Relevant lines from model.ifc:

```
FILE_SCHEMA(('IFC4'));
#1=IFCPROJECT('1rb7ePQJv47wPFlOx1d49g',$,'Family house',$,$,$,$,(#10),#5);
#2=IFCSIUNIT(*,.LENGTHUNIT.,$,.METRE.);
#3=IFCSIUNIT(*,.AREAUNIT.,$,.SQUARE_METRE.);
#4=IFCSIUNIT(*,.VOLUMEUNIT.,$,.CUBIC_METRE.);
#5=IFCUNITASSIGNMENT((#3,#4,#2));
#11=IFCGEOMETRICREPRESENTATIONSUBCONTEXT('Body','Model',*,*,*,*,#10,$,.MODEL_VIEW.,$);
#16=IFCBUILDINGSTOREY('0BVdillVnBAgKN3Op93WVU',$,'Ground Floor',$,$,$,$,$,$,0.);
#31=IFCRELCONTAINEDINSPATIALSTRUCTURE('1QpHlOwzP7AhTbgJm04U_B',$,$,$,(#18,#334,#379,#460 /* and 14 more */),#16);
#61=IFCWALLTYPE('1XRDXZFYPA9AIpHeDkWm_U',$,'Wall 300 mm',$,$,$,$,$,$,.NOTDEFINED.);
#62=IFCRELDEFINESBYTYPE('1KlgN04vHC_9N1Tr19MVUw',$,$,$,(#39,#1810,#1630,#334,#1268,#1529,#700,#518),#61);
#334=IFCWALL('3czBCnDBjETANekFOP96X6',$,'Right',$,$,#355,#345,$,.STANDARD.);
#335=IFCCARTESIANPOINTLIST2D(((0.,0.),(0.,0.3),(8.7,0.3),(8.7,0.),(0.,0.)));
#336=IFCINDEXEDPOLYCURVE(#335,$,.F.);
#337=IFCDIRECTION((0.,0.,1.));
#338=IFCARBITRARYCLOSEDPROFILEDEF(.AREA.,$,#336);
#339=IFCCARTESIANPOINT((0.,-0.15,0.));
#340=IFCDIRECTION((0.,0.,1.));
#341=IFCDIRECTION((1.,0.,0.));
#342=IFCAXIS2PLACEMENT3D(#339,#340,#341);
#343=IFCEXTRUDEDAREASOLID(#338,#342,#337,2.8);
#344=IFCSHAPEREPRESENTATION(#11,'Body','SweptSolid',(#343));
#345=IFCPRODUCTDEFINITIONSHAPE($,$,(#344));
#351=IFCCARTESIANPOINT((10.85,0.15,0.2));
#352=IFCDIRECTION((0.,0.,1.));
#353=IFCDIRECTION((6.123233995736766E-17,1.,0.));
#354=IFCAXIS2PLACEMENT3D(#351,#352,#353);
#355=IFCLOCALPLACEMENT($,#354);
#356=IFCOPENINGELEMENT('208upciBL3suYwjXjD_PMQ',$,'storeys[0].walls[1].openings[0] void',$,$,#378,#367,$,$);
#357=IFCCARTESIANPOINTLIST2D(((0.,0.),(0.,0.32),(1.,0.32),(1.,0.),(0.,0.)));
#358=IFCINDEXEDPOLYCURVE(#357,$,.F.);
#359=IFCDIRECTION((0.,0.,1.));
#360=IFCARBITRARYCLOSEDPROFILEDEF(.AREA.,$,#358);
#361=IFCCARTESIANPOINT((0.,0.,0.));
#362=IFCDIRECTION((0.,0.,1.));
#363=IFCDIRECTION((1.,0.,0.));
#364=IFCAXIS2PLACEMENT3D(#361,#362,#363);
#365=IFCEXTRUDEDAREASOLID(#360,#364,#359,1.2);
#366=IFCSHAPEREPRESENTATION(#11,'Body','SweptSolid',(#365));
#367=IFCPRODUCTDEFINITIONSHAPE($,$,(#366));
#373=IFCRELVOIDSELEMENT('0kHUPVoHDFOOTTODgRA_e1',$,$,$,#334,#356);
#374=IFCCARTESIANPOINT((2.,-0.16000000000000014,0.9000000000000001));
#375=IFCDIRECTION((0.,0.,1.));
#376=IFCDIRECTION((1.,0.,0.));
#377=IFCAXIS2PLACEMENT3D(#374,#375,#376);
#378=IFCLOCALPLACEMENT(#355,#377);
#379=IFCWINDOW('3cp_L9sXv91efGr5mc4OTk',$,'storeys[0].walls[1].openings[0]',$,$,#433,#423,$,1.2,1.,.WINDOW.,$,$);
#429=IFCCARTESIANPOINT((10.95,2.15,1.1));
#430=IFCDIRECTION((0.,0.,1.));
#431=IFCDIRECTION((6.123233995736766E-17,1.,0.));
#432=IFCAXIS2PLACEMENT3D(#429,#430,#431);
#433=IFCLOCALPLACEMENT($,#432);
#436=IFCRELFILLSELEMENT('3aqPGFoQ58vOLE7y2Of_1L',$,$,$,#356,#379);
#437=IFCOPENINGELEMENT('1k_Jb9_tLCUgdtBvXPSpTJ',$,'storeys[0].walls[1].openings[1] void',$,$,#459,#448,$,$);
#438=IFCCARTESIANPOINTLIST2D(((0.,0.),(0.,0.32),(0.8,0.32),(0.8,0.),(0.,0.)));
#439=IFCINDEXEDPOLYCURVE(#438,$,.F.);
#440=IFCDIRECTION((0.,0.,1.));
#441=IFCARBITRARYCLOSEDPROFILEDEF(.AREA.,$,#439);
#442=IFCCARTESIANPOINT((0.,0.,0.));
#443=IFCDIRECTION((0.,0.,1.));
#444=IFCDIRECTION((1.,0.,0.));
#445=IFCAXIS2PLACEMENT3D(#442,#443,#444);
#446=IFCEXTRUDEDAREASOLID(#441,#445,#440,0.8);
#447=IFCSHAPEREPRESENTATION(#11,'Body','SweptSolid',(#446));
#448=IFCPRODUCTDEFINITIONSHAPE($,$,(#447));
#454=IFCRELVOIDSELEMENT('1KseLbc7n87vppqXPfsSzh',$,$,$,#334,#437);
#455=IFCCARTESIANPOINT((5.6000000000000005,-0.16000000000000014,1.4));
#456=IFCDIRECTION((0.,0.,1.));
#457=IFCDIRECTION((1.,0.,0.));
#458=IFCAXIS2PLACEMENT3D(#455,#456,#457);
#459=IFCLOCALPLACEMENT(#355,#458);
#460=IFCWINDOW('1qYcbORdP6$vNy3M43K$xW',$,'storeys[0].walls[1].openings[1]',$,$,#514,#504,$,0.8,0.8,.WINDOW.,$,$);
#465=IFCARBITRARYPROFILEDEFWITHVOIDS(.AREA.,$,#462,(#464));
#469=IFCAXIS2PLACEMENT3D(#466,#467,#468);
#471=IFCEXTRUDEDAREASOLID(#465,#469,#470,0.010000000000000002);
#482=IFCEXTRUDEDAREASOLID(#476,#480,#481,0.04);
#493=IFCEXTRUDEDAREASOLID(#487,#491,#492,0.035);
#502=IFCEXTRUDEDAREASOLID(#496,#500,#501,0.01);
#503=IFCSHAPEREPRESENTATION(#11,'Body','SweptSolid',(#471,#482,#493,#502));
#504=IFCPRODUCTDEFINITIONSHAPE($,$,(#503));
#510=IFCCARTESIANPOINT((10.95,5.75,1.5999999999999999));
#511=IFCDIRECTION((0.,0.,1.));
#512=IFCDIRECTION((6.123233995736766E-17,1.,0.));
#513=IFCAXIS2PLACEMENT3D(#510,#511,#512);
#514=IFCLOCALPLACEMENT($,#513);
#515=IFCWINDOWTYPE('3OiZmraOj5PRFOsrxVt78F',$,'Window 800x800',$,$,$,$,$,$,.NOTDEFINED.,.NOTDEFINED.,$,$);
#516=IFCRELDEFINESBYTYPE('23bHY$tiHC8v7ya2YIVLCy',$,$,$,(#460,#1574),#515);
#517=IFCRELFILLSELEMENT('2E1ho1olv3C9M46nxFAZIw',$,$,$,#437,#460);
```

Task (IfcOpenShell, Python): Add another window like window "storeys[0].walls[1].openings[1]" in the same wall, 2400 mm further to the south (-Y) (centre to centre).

```python
import ifcopenshell
import ifcopenshell.api.feature
import ifcopenshell.api.geometry
import ifcopenshell.api.root
import ifcopenshell.geom
import ifcopenshell.util.element
import ifcopenshell.util.placement
import ifcopenshell.util.shape
import ifcopenshell.util.unit

model = ifcopenshell.open("model.ifc")
unit_scale = ifcopenshell.util.unit.calculate_unit_scale(model)
settings = ifcopenshell.geom.settings()


def volume(element):
    """Net volume in cubic metres, openings subtracted."""
    shape = ifcopenshell.geom.create_shape(settings, element)
    return ifcopenshell.util.shape.get_volume(shape.geometry)


window = model.by_id(460)
opening = window.FillsVoids[0].RelatingOpeningElement
wall = opening.VoidsElements[0].RelatingBuildingElement
before = volume(wall)
shift = ifcopenshell.util.placement.get_local_placement(wall.ObjectPlacement)[:3, 0] * -2.4 / unit_scale

# copy_class copies the void relationship, type, container and properties, but no geometry.
new_opening = ifcopenshell.api.root.copy_class(model, product=opening)
new_opening.Representation = ifcopenshell.util.element.copy_deep(
    model, opening.Representation, exclude=["IfcGeometricRepresentationContext", "IfcRepresentationMap"]
)
new_window = ifcopenshell.api.root.copy_class(model, product=window)
new_window.Representation = ifcopenshell.util.element.copy_deep(
    model, window.Representation, exclude=["IfcGeometricRepresentationContext", "IfcRepresentationMap"]
)
ifcopenshell.api.feature.add_filling(model, opening=new_opening, element=new_window)

for old, new in ((opening, new_opening), (window, new_window)):
    matrix = ifcopenshell.util.placement.get_local_placement(old.ObjectPlacement)
    matrix[:3, 3] += shift
    ifcopenshell.api.geometry.edit_object_placement(model, product=new, matrix=matrix, is_si=False)

after = volume(wall)

print(f"wall volume {before:.3f} -> {after:.3f} m3")

model.write("model_edited.ifc")
```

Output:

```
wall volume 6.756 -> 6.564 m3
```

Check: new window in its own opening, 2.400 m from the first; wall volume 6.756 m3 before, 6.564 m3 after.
